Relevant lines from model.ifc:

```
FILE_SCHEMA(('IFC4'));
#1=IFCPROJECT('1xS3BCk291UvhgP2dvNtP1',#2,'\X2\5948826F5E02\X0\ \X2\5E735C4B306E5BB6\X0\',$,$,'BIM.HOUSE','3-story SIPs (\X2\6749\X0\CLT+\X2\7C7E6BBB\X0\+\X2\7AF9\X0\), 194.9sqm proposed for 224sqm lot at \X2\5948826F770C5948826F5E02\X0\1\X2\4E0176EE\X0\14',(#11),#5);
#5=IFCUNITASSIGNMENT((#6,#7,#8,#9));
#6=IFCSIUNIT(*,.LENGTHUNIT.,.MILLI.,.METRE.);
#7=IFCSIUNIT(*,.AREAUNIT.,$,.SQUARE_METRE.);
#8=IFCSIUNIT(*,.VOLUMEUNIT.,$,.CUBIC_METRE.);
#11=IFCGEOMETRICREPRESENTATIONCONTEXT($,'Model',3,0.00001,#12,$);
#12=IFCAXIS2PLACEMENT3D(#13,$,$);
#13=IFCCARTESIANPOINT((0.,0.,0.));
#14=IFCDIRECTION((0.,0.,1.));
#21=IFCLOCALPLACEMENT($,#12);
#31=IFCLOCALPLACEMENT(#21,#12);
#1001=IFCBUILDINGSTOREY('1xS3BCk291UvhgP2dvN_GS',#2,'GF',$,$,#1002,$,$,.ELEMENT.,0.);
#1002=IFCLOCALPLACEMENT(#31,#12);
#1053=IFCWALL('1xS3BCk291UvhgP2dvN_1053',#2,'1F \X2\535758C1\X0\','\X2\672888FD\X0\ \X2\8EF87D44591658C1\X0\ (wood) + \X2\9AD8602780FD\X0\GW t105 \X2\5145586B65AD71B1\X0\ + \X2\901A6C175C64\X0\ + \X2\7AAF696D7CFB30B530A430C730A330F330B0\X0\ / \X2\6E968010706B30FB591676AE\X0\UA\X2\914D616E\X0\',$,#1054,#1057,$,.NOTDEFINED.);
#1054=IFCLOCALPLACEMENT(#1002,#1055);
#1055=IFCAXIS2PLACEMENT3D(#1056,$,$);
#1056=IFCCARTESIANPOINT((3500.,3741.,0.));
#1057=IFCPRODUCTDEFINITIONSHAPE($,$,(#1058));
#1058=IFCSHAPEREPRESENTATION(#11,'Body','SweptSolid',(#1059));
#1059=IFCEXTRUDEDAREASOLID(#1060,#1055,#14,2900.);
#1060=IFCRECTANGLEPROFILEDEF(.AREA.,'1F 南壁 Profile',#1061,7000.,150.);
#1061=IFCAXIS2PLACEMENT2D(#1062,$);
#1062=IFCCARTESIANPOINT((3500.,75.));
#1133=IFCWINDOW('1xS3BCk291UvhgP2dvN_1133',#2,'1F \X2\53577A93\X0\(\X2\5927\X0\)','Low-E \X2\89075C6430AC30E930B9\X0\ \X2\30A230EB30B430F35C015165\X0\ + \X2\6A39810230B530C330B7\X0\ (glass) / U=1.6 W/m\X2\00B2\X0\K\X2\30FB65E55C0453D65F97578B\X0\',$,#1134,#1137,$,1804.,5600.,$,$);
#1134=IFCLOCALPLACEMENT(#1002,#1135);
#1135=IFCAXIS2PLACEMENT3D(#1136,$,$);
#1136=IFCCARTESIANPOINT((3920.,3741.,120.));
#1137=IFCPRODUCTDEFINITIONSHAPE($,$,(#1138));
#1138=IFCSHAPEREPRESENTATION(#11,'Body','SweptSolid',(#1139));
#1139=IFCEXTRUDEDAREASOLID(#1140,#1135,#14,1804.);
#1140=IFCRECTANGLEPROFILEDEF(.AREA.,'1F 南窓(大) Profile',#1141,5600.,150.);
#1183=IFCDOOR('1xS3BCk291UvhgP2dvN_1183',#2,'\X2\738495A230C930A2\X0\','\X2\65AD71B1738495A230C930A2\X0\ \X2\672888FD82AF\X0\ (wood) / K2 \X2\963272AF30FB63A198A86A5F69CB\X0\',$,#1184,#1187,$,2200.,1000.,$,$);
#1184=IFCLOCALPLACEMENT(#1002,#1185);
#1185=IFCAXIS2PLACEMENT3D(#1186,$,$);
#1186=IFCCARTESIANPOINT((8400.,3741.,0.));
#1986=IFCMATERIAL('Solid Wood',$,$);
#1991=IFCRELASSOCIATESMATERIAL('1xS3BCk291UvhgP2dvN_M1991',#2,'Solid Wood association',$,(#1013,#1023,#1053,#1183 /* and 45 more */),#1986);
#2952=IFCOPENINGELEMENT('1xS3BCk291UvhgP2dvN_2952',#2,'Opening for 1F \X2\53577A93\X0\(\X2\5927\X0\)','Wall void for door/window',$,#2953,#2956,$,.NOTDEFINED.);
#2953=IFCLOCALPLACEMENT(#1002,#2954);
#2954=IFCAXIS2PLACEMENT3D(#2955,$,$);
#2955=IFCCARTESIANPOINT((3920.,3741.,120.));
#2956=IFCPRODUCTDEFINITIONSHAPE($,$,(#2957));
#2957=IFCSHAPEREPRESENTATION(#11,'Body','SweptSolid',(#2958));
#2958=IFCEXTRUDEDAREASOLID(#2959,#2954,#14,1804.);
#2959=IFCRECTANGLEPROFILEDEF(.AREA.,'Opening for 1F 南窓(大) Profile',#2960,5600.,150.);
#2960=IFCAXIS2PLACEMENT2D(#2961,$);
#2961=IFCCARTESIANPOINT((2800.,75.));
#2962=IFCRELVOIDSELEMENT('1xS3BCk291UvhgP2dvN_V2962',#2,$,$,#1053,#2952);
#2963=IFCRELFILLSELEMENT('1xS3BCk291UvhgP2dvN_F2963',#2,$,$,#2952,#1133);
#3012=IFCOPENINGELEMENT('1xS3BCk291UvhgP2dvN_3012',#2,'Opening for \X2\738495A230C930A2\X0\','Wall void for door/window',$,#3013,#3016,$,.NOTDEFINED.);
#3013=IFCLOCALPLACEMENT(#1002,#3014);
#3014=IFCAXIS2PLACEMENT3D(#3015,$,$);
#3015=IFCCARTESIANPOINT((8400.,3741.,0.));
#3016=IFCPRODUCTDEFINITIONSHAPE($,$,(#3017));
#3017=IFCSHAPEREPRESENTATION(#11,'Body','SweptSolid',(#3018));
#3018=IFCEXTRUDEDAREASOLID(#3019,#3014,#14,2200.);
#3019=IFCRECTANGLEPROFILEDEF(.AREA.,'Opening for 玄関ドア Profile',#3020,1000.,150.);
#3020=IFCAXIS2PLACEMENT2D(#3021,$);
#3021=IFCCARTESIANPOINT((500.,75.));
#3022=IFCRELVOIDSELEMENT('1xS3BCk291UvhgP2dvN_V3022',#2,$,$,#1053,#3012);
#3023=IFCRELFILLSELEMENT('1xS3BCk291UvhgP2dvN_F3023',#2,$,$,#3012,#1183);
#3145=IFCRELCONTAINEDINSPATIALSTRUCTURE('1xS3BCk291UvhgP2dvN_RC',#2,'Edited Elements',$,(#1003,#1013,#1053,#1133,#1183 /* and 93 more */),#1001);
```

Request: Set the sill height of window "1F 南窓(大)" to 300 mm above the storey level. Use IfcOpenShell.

```python
import numpy as np
import ifcopenshell
import ifcopenshell.api.geometry
import ifcopenshell.geom
import ifcopenshell.util.element
import ifcopenshell.util.placement
import ifcopenshell.util.shape
import ifcopenshell.util.unit

model = ifcopenshell.open("model.ifc")
unit_scale = ifcopenshell.util.unit.calculate_unit_scale(model)

window = model.by_guid("1xS3BCk291UvhgP2dvN_1133")
opening = window.FillsVoids[0].RelatingOpeningElement
storey = ifcopenshell.util.element.get_container(window, ifc_class="IfcBuildingStorey")
level = ifcopenshell.util.placement.get_local_placement(storey.ObjectPlacement)[2, 3]

# The opening's origin need not be at the sill, so measure its lowest point.
shape = ifcopenshell.geom.create_shape(ifcopenshell.geom.settings(), opening)
bottom = ifcopenshell.util.shape.get_shape_bottom_elevation(shape, shape.geometry) / unit_scale
dz = level + 0.3 / unit_scale - bottom

shift = np.array([0.0, 0.0, dz])
# The window is not placed relative to its opening, so move both.
for product in (opening, window):
    matrix = ifcopenshell.util.placement.get_local_placement(product.ObjectPlacement)
    matrix[:3, 3] += shift
    ifcopenshell.api.geometry.edit_object_placement(model, product=product, matrix=matrix, is_si=False)

print(f"moved by {dz * unit_scale:+.3f} m")

model.write("model-out.ifc")
```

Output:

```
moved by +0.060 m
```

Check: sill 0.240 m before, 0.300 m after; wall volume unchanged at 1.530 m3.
